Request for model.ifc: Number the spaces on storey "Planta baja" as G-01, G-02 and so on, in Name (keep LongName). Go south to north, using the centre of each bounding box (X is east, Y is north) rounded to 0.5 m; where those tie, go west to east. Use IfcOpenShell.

First a look at what the model holds.

```python
import ifcopenshell
import ifcopenshell.util.element
import ifcopenshell.util.placement

model = ifcopenshell.open("model.ifc")
print(model.schema)
storey = next(s for s in model.by_type("IfcBuildingStorey") if s.Name == "Planta baja")
spaces = [e for e in ifcopenshell.util.element.get_decomposition(storey) if e.is_a("IfcSpace")]
for e in sorted(spaces, key=lambda e: e.id()):
    origin = ifcopenshell.util.placement.get_local_placement(e.ObjectPlacement)[:3, 3]
    print(e.id(), e.Name, e.LongName, origin.round(2) + 0.0, sep=" | ")
```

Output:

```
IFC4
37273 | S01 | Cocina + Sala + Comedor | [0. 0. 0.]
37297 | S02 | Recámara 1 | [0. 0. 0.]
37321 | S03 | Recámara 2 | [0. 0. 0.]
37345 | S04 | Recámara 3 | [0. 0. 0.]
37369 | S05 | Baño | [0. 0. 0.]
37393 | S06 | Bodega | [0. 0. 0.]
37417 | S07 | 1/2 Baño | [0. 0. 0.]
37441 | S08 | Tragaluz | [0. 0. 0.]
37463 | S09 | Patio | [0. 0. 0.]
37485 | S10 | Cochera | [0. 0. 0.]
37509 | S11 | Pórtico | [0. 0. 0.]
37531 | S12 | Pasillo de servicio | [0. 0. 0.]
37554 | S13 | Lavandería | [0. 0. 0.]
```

```python
import ifcopenshell
import ifcopenshell.geom
import ifcopenshell.util.element
import ifcopenshell.util.shape

model = ifcopenshell.open("model.ifc")
settings = ifcopenshell.geom.settings()
settings.set("use-world-coords", True)


def centre(element):
    shape = ifcopenshell.geom.create_shape(settings, element)
    return ifcopenshell.util.shape.get_bbox_centroid(shape.geometry)


storey = next(s for s in model.by_type("IfcBuildingStorey") if s.Name == "Planta baja")
spaces = [e for e in ifcopenshell.util.element.get_decomposition(storey) if e.is_a("IfcSpace")]

# Insertion points can sit at a corner or the storey origin, so sort by the geometry (in metres).
centres = {e: centre(e) for e in spaces}
spaces.sort(key=lambda e: (round(centres[e][1] / 0.5), centres[e][0]))

for i, e in enumerate(spaces, start=1):
    number = f"G-{i:02d}"
    e.Name = number
    print(e.id(), number)

model.write("model_edited.ifc")
```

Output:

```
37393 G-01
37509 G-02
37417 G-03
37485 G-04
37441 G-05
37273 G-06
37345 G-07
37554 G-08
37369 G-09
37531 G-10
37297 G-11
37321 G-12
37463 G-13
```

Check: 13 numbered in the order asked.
